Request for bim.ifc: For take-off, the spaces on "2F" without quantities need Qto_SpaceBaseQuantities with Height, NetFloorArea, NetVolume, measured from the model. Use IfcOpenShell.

First a look at what the model holds.

```python
import ifcopenshell
import ifcopenshell.util.element
import ifcopenshell.util.unit

model = ifcopenshell.open("bim.ifc")
print(model.schema)
for unit_type in ("LENGTHUNIT", "AREAUNIT", "VOLUMEUNIT"):
    print(unit_type, ifcopenshell.util.unit.calculate_unit_scale(model, unit_type))
storey = next(s for s in model.by_type("IfcBuildingStorey") if s.Name == "2F")
spaces = [e for e in ifcopenshell.util.element.get_decomposition(storey) if e.is_a("IfcSpace")]
for e in sorted(spaces, key=lambda e: e.id()):
    print(e.id(), e.is_a(), e.Name, list(ifcopenshell.util.element.get_psets(e, qtos_only=True)), sep=" | ")
```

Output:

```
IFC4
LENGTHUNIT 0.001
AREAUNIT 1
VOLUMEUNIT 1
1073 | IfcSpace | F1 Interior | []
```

```python
import ifcopenshell
import ifcopenshell.api.pset
import ifcopenshell.geom
import ifcopenshell.util.element
import ifcopenshell.util.shape
import ifcopenshell.util.unit

model = ifcopenshell.open("bim.ifc")
unit_scale = ifcopenshell.util.unit.calculate_unit_scale(model)
area_scale = ifcopenshell.util.unit.calculate_unit_scale(model, "AREAUNIT")
volume_scale = ifcopenshell.util.unit.calculate_unit_scale(model, "VOLUMEUNIT")
settings = ifcopenshell.geom.settings()

storey = next(s for s in model.by_type("IfcBuildingStorey") if s.Name == "2F")
spaces = [e for e in ifcopenshell.util.element.get_decomposition(storey) if e.is_a("IfcSpace")]

for e in sorted(spaces, key=lambda e: e.id()):
    if ifcopenshell.util.element.get_psets(e, qtos_only=True, should_inherit=False):
        continue
    # Geometry comes back in metres, in the element's own axes.
    shape = ifcopenshell.geom.create_shape(settings, e)
    values = {
        "Height": ifcopenshell.util.shape.get_z(shape.geometry) / unit_scale,
        "NetFloorArea": ifcopenshell.util.shape.get_footprint_area(shape.geometry) / area_scale,
        "NetVolume": ifcopenshell.util.shape.get_volume(shape.geometry) / volume_scale,
    }
    qto = ifcopenshell.api.pset.add_qto(model, product=e, name="Qto_SpaceBaseQuantities")
    ifcopenshell.api.pset.edit_qto(model, qto=qto, properties=values)
    print(e.id(), {k: round(v, 3) for k, v in values.items()})

model.write("bim_v2.ifc")
```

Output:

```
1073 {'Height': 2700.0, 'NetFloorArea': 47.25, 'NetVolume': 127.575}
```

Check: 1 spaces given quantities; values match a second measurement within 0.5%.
